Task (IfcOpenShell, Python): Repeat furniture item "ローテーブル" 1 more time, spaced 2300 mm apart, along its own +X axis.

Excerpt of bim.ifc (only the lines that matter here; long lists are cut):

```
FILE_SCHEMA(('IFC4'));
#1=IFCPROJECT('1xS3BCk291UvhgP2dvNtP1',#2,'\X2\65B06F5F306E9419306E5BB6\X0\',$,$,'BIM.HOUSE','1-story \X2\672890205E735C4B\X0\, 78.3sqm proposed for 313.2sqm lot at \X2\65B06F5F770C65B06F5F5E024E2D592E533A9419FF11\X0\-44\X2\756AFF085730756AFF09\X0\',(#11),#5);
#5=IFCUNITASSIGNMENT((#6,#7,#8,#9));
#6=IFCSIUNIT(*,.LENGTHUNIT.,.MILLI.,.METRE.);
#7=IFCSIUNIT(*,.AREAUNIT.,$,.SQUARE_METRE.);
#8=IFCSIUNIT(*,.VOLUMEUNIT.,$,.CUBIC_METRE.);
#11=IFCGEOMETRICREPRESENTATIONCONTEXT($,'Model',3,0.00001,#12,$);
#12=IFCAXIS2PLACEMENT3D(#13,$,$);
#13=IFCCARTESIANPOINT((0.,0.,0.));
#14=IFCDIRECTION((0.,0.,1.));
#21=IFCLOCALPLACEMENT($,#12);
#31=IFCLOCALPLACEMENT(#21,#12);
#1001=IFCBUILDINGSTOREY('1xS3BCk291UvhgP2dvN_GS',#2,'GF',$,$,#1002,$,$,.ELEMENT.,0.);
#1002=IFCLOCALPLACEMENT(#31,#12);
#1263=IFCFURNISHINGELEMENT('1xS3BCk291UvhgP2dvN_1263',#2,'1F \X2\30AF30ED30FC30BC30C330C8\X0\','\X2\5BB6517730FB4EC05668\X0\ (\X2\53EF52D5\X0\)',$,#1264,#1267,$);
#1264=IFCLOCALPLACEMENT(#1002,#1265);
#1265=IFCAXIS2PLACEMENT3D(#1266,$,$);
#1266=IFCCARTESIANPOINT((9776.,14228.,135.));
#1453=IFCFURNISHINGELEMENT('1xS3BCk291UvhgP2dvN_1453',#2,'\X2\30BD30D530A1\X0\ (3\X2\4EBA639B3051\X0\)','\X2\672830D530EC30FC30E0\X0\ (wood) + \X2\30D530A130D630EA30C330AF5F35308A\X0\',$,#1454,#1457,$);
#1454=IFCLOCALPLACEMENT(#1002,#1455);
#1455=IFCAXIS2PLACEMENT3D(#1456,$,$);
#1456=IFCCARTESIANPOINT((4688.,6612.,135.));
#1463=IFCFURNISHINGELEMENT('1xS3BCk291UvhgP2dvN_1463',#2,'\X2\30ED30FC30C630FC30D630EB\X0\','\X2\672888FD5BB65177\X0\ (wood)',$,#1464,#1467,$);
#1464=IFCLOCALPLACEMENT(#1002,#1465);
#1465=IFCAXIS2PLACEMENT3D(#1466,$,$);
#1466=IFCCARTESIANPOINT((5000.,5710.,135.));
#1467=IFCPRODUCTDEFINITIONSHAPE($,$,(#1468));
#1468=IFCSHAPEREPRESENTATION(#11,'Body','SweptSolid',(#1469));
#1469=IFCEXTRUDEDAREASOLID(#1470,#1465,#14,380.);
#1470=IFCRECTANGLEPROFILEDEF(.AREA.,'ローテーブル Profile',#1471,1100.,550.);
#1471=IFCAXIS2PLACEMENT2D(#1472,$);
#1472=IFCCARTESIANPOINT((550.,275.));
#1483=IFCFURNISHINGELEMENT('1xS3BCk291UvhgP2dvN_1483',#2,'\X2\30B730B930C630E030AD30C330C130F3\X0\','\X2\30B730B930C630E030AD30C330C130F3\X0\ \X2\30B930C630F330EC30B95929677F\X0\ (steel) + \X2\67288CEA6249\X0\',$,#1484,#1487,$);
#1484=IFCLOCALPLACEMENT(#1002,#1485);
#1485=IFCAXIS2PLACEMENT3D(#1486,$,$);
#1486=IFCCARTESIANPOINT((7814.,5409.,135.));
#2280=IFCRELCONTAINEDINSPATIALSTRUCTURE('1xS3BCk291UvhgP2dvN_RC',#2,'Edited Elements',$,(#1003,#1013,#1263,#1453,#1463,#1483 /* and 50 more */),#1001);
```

```python
import ifcopenshell
import ifcopenshell.api.geometry
import ifcopenshell.api.root
import ifcopenshell.util.element
import ifcopenshell.util.placement

model = ifcopenshell.open("bim.ifc")


def reuse_history(source, copy):
    """copy_class also copies each property set's owner history, people and application; keep the originals."""
    for rel in copy.IsDefinedBy:
        if rel.is_a("IfcRelDefinesByProperties") and (history := rel.RelatingPropertyDefinition.OwnerHistory):
            rel.RelatingPropertyDefinition.OwnerHistory = source.OwnerHistory
            ifcopenshell.util.element.remove_deep2(model, history)


source = model.by_guid("1xS3BCk291UvhgP2dvN_1463")
base = ifcopenshell.util.placement.get_local_placement(source.ObjectPlacement)
step = base[:3, 0] * 2300.0

for i in range(1, 2):
    copy = ifcopenshell.api.root.copy_class(model, product=source)
    copy.Representation = ifcopenshell.util.element.copy_deep(
        model, source.Representation, exclude=["IfcGeometricRepresentationContext", "IfcRepresentationMap"]
    )
    reuse_history(source, copy)
    matrix = base.copy()
    matrix[:3, 3] += i * step
    print("added at", matrix[:3, 3].round(3) + 0.0)
    ifcopenshell.api.geometry.edit_object_placement(model, product=copy, matrix=matrix, is_si=False)

model.write("bim_v2.ifc")
```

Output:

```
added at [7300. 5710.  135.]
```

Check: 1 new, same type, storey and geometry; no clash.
